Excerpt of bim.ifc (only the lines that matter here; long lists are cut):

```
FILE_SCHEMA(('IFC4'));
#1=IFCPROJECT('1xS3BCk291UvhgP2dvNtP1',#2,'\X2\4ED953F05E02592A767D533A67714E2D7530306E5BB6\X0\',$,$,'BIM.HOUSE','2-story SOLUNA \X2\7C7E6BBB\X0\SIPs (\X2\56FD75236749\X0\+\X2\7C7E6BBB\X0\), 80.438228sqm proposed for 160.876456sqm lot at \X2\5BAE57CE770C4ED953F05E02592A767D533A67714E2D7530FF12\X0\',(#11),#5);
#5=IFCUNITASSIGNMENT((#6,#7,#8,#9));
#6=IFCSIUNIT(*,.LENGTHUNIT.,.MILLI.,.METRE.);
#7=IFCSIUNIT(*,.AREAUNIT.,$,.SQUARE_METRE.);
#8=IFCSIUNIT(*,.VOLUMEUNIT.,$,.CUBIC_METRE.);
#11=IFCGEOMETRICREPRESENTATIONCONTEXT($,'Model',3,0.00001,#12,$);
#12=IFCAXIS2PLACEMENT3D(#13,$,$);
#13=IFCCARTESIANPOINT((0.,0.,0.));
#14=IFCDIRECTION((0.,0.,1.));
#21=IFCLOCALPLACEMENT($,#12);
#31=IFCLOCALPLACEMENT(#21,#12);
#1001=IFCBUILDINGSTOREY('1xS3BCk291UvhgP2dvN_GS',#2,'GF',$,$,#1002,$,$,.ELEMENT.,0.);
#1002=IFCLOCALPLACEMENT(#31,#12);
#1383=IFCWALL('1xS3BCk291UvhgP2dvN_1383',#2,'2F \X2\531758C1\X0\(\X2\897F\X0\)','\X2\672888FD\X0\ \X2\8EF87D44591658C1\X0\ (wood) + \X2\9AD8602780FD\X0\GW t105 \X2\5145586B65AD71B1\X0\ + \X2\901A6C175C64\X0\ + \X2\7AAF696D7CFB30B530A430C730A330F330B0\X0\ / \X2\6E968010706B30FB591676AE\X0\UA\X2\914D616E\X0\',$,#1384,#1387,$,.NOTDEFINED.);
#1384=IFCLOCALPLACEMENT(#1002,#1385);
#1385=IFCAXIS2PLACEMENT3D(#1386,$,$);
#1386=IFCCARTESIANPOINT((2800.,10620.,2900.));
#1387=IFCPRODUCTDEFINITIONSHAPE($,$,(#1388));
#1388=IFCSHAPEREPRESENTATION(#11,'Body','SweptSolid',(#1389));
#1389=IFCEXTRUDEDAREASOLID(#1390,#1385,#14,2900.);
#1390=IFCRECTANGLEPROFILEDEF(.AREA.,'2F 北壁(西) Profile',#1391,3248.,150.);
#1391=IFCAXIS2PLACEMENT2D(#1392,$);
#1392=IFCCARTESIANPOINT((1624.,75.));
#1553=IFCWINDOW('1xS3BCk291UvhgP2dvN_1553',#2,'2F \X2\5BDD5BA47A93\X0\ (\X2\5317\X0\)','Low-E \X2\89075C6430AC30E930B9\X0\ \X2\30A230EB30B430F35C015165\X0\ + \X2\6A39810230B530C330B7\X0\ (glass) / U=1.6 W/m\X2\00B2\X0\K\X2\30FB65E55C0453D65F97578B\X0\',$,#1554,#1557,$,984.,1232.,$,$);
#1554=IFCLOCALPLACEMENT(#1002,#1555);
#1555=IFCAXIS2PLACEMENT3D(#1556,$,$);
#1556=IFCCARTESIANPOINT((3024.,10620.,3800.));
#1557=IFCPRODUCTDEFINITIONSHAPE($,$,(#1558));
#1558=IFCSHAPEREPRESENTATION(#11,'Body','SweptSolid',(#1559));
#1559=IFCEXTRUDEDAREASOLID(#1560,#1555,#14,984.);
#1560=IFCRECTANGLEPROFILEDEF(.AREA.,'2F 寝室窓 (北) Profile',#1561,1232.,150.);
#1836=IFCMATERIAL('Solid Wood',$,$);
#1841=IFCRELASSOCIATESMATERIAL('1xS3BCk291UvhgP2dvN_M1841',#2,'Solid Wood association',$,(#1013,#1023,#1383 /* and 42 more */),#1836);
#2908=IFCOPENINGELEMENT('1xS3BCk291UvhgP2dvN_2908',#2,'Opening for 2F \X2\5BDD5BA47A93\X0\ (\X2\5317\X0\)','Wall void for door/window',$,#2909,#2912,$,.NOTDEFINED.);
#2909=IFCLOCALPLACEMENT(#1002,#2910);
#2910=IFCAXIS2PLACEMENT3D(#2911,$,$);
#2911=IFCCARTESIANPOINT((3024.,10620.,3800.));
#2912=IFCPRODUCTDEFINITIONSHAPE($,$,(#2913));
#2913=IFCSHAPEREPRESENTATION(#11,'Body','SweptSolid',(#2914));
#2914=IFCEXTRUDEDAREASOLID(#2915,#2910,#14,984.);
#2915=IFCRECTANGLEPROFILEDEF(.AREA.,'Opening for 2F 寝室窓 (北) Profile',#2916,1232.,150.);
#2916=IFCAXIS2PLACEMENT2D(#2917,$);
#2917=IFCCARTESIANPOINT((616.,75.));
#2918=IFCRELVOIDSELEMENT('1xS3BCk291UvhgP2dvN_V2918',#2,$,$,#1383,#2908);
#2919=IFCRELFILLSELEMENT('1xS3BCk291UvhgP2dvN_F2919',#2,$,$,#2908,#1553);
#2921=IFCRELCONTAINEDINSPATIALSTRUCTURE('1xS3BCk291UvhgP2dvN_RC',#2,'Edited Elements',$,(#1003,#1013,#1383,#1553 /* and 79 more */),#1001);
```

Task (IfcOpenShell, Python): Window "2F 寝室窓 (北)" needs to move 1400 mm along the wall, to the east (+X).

```python
import ifcopenshell
import ifcopenshell.api.geometry
import ifcopenshell.util.placement
import ifcopenshell.util.unit

model = ifcopenshell.open("bim.ifc")
unit_scale = ifcopenshell.util.unit.calculate_unit_scale(model)

window = model.by_id(1553)
opening = window.FillsVoids[0].RelatingOpeningElement
wall = opening.VoidsElements[0].RelatingBuildingElement

wall_matrix = ifcopenshell.util.placement.get_local_placement(wall.ObjectPlacement)
shift = wall_matrix[:3, 0] * 1.4 / unit_scale
before = ifcopenshell.util.placement.get_local_placement(window.ObjectPlacement)[:3, 3].copy()

# The window is not placed relative to its opening, so move both.
for product in (opening, window):
    matrix = ifcopenshell.util.placement.get_local_placement(product.ObjectPlacement)
    matrix[:3, 3] += shift
    ifcopenshell.api.geometry.edit_object_placement(model, product=product, matrix=matrix, is_si=False)

after = ifcopenshell.util.placement.get_local_placement(window.ObjectPlacement)[:3, 3]
print("window moved by", (after - before).round(3) + 0.0)

model.write("bim_rev.ifc")
```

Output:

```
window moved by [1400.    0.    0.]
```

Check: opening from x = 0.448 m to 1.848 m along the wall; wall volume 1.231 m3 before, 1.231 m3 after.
